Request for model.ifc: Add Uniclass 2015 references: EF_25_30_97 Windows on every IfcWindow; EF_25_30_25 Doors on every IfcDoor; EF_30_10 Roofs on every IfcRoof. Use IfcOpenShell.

First a look at what the model holds.

```python
import ifcopenshell

model = ifcopenshell.open("model.ifc")
print(model.schema)
print("classifications:", [c.Name for c in model.by_type("IfcClassification")])
for ifc_class in ("IfcDoor", "IfcRoof", "IfcStair", "IfcWall", "IfcWindow"):
    print(ifc_class, len(model.by_type(ifc_class)))
```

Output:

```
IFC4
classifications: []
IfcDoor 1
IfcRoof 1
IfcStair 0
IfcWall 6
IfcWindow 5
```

```python
import ifcopenshell
import ifcopenshell.api.classification

model = ifcopenshell.open("model.ifc")

system = ifcopenshell.api.classification.add_classification(model, classification="Uniclass 2015")

codes = {
    "IfcWindow": ("EF_25_30_97", "Windows"),
    "IfcDoor": ("EF_25_30_25", "Doors"),
    "IfcRoof": ("EF_30_10", "Roofs"),
}
for ifc_class, (code, name) in codes.items():
    products = model.by_type(ifc_class)
    ifcopenshell.api.classification.add_reference(
        model, products=products, classification=system, identification=code, name=name
    )
    print(code, len(products))

model.write("model_edited.ifc")
```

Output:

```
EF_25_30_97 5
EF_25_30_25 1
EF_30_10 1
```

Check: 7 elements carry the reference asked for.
